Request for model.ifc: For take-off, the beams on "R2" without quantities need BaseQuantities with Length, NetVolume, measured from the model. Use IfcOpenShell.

First a look at what the model holds.

```python
import ifcopenshell
import ifcopenshell.util.element
import ifcopenshell.util.unit

model = ifcopenshell.open("model.ifc")
print(model.schema)
for unit_type in ("LENGTHUNIT", "AREAUNIT", "VOLUMEUNIT"):
    print(unit_type, ifcopenshell.util.unit.calculate_unit_scale(model, unit_type))
storey = next(s for s in model.by_type("IfcBuildingStorey") if s.Name == "R2")
beams = [e for e in ifcopenshell.util.element.get_decomposition(storey) if e.is_a("IfcBeam")]
for e in sorted(beams, key=lambda e: e.id()):
    print(e.id(), e.is_a(), e.Name, list(ifcopenshell.util.element.get_psets(e, qtos_only=True)), sep=" | ")
```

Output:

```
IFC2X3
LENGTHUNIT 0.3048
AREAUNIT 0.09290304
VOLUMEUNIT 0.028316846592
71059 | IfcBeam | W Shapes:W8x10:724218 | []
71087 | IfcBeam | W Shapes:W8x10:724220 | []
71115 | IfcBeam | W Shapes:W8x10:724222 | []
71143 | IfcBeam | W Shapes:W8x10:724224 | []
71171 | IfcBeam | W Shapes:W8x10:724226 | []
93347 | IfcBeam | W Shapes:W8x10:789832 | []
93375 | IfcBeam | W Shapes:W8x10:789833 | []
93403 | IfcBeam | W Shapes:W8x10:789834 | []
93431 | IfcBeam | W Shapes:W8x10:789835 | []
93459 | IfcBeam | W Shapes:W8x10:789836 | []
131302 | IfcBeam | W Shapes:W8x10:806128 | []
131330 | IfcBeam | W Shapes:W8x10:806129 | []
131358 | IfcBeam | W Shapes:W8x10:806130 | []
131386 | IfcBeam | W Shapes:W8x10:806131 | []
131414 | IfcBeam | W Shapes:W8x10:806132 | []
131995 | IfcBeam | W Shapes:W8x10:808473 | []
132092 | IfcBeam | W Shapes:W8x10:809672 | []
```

```python
import ifcopenshell
import ifcopenshell.api.pset
import ifcopenshell.geom
import ifcopenshell.util.element
import ifcopenshell.util.shape
import ifcopenshell.util.unit

model = ifcopenshell.open("model.ifc")
unit_scale = ifcopenshell.util.unit.calculate_unit_scale(model)
volume_scale = ifcopenshell.util.unit.calculate_unit_scale(model, "VOLUMEUNIT")
settings = ifcopenshell.geom.settings()

storey = next(s for s in model.by_type("IfcBuildingStorey") if s.Name == "R2")
beams = [e for e in ifcopenshell.util.element.get_decomposition(storey) if e.is_a("IfcBeam")]

for e in sorted(beams, key=lambda e: e.id()):
    if ifcopenshell.util.element.get_psets(e, qtos_only=True, should_inherit=False):
        continue
    # Geometry comes back in metres, in the element's own axes.
    shape = ifcopenshell.geom.create_shape(settings, e)
    values = {
        "Length": ifcopenshell.util.shape.get_max_xyz(shape.geometry) / unit_scale,
        "NetVolume": ifcopenshell.util.shape.get_volume(shape.geometry) / volume_scale,
    }
    qto = ifcopenshell.api.pset.add_qto(model, product=e, name="BaseQuantities")
    ifcopenshell.api.pset.edit_qto(model, qto=qto, properties=values)
    print(e.id(), {k: round(v, 3) for k, v in values.items()})

model.write("model-out.ifc")
```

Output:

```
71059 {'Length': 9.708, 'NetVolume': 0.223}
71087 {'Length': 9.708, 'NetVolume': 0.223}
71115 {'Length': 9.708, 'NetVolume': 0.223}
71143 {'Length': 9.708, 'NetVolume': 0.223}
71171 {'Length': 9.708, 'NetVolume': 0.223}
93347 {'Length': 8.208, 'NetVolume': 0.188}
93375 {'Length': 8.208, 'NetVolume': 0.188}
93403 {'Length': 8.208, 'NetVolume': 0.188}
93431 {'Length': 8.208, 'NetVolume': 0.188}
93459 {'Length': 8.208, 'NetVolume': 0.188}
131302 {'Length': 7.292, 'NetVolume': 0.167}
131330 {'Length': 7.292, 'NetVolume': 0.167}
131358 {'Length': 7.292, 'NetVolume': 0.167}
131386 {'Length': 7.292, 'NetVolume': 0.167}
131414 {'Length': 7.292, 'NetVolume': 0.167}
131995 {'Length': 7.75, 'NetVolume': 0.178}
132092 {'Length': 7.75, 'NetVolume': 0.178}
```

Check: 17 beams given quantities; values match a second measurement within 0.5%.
